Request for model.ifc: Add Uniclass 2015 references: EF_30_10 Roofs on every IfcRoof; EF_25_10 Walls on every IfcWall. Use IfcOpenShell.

First a look at what the model holds.

```python
import ifcopenshell

model = ifcopenshell.open("model.ifc")
print(model.schema)
print("classifications:", [c.Name for c in model.by_type("IfcClassification")])
for ifc_class in ("IfcDoor", "IfcRoof", "IfcStair", "IfcWall", "IfcWindow"):
    print(ifc_class, len(model.by_type(ifc_class)))
```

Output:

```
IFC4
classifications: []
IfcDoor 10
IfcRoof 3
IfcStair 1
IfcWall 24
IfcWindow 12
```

```python
import ifcopenshell
import ifcopenshell.api.classification

model = ifcopenshell.open("model.ifc")

system = ifcopenshell.api.classification.add_classification(model, classification="Uniclass 2015")

codes = {
    "IfcRoof": ("EF_30_10", "Roofs"),
    "IfcWall": ("EF_25_10", "Walls"),
}
for ifc_class, (code, name) in codes.items():
    products = model.by_type(ifc_class)
    ifcopenshell.api.classification.add_reference(
        model, products=products, classification=system, identification=code, name=name
    )
    print(code, len(products))

model.write("model_v2.ifc")
```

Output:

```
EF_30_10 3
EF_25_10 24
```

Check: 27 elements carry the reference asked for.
